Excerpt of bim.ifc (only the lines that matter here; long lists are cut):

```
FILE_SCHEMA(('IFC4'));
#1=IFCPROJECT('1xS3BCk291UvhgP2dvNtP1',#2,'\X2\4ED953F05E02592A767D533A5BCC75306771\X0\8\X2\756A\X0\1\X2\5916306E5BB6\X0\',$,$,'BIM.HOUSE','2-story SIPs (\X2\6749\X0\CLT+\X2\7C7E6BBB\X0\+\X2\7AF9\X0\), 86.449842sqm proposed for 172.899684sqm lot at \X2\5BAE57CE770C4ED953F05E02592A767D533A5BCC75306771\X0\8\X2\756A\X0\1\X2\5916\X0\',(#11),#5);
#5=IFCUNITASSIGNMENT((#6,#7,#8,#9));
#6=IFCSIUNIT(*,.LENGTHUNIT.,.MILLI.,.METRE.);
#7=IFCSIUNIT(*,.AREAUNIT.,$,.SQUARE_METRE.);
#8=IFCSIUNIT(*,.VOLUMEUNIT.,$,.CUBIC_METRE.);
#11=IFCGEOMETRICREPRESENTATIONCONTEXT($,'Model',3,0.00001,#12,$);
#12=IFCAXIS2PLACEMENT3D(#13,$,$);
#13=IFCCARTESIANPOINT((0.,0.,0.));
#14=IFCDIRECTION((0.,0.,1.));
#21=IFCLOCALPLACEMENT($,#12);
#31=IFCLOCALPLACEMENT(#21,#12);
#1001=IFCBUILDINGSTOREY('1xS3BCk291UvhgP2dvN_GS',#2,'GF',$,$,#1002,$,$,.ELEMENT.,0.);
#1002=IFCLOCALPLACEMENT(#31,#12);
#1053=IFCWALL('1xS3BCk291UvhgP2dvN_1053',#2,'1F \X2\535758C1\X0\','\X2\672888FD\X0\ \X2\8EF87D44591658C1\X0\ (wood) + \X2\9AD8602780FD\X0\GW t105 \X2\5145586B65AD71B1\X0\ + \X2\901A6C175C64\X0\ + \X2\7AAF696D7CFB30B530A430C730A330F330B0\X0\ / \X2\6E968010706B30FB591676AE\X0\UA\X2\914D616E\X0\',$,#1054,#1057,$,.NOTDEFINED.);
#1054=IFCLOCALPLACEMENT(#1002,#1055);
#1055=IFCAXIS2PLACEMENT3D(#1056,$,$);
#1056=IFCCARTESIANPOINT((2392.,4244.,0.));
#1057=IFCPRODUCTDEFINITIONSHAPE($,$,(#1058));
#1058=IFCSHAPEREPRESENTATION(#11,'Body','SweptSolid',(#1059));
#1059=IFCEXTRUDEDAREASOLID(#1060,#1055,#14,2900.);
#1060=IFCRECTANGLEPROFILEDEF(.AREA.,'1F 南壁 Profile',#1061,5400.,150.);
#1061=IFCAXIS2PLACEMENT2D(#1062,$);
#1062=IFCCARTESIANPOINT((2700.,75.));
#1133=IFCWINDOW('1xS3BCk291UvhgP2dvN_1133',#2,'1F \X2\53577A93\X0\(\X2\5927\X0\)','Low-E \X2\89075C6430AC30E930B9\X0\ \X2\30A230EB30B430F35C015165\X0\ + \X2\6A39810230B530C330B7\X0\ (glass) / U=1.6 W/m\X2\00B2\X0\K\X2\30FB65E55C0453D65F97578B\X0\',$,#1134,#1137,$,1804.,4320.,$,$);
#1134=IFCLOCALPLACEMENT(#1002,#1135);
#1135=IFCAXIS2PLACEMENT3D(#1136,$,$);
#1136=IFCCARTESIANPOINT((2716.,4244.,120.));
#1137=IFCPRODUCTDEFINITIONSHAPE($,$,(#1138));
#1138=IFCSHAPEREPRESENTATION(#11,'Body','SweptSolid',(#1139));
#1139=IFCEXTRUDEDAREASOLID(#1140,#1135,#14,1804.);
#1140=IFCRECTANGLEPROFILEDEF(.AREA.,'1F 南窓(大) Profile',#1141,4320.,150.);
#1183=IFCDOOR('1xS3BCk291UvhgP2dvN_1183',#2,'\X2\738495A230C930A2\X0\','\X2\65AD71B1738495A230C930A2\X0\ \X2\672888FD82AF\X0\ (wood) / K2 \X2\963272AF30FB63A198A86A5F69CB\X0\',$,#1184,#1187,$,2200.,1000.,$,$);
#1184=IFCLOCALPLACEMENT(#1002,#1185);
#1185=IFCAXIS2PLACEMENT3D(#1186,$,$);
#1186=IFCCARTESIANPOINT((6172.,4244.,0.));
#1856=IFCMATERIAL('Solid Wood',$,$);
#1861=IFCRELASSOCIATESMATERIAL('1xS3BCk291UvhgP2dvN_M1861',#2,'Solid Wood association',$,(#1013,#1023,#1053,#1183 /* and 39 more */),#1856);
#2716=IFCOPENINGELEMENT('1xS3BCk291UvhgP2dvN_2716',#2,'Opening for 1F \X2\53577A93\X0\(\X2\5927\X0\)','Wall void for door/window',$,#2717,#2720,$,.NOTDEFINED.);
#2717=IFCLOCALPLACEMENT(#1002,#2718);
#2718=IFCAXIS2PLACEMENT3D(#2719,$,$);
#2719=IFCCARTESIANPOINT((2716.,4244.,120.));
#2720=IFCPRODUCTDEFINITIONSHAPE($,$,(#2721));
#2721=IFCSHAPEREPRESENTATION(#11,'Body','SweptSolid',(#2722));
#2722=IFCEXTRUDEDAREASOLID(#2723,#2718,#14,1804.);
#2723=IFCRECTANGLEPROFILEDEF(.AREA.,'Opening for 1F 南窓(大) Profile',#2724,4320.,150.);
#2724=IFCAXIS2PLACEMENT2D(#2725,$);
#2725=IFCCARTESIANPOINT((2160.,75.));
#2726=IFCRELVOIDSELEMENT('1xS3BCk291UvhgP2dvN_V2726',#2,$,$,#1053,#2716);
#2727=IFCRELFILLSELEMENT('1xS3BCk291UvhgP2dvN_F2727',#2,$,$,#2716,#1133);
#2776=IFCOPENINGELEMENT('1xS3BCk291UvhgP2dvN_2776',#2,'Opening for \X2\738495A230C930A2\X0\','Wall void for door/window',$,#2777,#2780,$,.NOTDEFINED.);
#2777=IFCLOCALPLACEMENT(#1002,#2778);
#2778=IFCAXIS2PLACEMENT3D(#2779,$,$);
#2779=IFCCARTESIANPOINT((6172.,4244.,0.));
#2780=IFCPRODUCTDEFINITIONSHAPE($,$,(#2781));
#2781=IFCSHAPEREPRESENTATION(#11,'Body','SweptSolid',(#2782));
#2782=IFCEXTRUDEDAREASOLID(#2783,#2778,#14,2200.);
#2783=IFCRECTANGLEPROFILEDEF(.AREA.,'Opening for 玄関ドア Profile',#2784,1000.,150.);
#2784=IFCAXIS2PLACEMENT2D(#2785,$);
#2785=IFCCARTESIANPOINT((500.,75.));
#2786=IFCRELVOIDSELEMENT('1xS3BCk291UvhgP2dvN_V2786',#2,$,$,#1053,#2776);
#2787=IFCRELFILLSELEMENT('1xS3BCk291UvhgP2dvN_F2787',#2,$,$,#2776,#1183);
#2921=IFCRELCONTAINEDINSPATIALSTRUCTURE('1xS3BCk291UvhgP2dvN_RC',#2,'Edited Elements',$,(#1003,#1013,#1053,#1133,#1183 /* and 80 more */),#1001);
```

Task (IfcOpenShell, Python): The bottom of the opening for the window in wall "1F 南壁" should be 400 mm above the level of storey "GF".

```python
import numpy as np
import ifcopenshell
import ifcopenshell.api.geometry
import ifcopenshell.geom
import ifcopenshell.util.element
import ifcopenshell.util.placement
import ifcopenshell.util.shape
import ifcopenshell.util.unit

model = ifcopenshell.open("bim.ifc")
unit_scale = ifcopenshell.util.unit.calculate_unit_scale(model)

window = model.by_id(1133)
opening = window.FillsVoids[0].RelatingOpeningElement
storey = ifcopenshell.util.element.get_container(window, ifc_class="IfcBuildingStorey")
level = ifcopenshell.util.placement.get_local_placement(storey.ObjectPlacement)[2, 3]

# The opening's origin need not be at the sill, so measure its lowest point.
shape = ifcopenshell.geom.create_shape(ifcopenshell.geom.settings(), opening)
bottom = ifcopenshell.util.shape.get_shape_bottom_elevation(shape, shape.geometry) / unit_scale
dz = level + 0.4 / unit_scale - bottom

shift = np.array([0.0, 0.0, dz])
# The window is not placed relative to its opening, so move both.
for product in (opening, window):
    matrix = ifcopenshell.util.placement.get_local_placement(product.ObjectPlacement)
    matrix[:3, 3] += shift
    ifcopenshell.api.geometry.edit_object_placement(model, product=product, matrix=matrix, is_si=False)

print(f"moved by {dz * unit_scale:+.3f} m")

model.write("bim_edited.ifc")
```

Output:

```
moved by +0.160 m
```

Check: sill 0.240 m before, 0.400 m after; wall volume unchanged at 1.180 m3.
